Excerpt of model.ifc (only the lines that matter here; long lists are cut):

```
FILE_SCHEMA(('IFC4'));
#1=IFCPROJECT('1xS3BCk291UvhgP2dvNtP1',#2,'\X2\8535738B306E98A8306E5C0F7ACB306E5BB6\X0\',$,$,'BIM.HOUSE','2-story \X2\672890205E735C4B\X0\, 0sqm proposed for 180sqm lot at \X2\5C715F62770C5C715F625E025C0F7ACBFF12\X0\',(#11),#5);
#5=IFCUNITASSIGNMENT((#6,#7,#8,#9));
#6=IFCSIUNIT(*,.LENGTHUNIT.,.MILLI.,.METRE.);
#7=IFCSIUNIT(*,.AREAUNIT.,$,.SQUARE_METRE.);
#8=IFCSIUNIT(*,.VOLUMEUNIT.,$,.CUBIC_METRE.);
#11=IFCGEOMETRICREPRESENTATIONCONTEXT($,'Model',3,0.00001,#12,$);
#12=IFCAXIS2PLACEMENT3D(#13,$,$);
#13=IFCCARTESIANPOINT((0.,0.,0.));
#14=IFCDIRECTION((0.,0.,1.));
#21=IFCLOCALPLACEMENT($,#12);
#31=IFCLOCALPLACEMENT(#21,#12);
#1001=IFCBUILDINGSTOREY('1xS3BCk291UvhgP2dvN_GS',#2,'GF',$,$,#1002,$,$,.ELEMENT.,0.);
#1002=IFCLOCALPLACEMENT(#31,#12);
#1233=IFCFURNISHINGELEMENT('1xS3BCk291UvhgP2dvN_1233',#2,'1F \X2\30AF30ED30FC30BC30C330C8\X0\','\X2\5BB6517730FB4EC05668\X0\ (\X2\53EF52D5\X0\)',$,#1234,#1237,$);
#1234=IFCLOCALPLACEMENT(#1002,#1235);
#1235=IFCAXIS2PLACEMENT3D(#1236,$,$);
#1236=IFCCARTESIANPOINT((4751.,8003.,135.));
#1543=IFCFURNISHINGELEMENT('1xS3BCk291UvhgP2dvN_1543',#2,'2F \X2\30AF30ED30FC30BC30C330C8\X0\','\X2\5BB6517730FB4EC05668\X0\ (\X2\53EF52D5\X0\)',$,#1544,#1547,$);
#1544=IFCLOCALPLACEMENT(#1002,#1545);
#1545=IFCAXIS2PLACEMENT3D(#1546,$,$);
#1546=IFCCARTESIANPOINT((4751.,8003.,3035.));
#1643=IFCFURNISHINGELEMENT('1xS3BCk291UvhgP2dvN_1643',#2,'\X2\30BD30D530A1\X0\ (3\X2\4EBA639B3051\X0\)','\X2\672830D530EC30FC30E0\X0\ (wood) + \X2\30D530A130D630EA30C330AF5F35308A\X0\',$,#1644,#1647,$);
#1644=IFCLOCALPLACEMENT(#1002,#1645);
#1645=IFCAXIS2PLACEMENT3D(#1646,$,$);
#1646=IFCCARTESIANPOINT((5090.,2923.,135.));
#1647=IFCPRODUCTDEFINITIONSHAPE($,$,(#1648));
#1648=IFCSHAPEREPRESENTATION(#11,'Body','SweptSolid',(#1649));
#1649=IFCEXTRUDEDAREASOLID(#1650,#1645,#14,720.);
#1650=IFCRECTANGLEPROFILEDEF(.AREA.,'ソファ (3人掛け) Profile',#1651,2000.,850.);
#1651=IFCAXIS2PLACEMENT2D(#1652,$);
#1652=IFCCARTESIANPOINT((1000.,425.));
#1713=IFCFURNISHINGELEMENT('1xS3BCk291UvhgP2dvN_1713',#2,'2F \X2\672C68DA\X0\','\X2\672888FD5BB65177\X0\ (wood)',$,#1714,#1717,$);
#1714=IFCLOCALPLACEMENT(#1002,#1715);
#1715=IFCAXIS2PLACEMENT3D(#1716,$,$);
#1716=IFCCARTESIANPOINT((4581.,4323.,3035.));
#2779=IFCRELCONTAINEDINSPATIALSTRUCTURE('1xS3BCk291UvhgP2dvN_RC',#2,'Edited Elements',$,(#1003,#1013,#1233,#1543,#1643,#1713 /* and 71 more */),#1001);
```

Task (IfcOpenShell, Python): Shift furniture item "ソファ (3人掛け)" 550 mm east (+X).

```python
import ifcopenshell
import ifcopenshell.api.geometry
import ifcopenshell.util.placement

model = ifcopenshell.open("model.ifc")

item = model.by_guid("1xS3BCk291UvhgP2dvN_1643")
matrix = ifcopenshell.util.placement.get_local_placement(item.ObjectPlacement)
matrix[0, 3] += 550.0
ifcopenshell.api.geometry.edit_object_placement(model, product=item, matrix=matrix, is_si=False)

print(ifcopenshell.util.placement.get_local_placement(item.ObjectPlacement).round(3) + 0.0)

model.write("model-out.ifc")
```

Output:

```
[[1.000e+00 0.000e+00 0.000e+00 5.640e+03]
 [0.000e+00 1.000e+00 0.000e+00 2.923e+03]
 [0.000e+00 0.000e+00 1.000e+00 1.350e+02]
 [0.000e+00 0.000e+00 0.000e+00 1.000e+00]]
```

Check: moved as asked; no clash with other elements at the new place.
